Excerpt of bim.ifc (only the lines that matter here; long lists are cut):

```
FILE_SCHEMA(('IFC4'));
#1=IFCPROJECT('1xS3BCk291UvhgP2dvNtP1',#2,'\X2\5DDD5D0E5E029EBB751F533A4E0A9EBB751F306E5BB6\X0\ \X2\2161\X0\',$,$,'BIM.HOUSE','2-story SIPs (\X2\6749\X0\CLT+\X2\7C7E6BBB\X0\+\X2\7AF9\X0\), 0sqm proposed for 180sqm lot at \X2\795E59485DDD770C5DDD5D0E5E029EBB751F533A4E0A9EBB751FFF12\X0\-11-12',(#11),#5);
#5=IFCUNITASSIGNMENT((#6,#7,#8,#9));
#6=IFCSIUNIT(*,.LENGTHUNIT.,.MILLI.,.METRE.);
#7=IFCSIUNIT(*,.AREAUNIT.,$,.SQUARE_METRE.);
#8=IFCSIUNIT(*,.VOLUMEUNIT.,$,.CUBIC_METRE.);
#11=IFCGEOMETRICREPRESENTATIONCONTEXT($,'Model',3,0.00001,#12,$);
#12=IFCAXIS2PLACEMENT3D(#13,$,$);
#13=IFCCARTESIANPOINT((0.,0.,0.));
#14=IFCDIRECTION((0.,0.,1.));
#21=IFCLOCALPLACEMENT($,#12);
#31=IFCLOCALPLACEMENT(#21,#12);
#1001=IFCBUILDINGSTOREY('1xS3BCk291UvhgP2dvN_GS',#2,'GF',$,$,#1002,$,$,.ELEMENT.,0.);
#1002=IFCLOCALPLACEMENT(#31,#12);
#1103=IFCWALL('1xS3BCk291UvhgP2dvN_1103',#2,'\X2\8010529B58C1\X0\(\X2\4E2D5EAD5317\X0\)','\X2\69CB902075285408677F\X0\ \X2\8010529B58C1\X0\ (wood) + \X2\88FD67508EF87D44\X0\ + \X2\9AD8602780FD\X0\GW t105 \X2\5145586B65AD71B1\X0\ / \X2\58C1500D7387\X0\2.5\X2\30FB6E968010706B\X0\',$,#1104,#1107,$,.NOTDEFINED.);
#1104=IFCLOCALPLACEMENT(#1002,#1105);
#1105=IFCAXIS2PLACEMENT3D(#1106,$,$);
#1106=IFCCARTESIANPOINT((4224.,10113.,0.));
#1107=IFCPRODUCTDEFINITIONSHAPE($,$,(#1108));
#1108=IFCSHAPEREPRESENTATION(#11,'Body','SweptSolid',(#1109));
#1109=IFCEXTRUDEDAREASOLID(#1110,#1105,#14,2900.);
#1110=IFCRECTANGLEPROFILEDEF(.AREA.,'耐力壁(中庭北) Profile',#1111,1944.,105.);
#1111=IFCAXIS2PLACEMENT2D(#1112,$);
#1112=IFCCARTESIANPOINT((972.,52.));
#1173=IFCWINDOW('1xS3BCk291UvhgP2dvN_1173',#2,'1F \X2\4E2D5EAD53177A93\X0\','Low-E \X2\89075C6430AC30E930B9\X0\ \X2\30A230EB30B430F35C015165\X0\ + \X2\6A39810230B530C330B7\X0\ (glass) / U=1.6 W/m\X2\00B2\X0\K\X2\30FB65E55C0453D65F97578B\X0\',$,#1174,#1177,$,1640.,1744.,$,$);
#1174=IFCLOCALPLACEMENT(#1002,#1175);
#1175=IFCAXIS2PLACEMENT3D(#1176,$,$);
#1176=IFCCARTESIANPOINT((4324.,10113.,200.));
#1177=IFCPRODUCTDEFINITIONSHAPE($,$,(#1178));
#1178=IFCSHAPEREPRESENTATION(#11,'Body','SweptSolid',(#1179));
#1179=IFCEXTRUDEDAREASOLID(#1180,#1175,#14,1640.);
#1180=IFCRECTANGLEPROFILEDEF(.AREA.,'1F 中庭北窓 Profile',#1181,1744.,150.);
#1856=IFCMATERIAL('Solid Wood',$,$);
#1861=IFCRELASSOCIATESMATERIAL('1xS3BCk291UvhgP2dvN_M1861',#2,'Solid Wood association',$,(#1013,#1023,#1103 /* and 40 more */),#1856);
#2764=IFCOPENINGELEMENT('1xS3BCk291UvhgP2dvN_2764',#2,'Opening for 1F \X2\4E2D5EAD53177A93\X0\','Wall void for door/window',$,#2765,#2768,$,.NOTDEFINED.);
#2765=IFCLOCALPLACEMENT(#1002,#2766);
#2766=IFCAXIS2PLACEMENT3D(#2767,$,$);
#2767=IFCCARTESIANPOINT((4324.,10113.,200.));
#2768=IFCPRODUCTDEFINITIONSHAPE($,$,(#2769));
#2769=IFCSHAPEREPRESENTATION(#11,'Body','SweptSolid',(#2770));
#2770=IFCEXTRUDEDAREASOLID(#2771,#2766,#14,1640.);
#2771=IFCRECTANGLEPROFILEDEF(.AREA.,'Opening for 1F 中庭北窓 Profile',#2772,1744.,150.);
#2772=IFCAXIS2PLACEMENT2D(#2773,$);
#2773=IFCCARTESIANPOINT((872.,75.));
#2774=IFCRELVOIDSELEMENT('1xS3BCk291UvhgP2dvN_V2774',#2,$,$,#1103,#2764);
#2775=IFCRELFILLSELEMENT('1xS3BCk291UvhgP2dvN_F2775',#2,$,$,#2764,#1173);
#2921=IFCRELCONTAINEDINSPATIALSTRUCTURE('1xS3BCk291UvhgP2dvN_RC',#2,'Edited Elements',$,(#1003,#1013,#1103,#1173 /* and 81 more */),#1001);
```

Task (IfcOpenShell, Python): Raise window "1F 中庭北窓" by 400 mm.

```python
import numpy as np
import ifcopenshell
import ifcopenshell.api.geometry
import ifcopenshell.util.placement
import ifcopenshell.util.unit

model = ifcopenshell.open("bim.ifc")
unit_scale = ifcopenshell.util.unit.calculate_unit_scale(model)

window = model.by_guid("1xS3BCk291UvhgP2dvN_1173")
opening = window.FillsVoids[0].RelatingOpeningElement
dz = 0.4 / unit_scale

shift = np.array([0.0, 0.0, dz])
# The window is not placed relative to its opening, so move both.
for product in (opening, window):
    matrix = ifcopenshell.util.placement.get_local_placement(product.ObjectPlacement)
    matrix[:3, 3] += shift
    ifcopenshell.api.geometry.edit_object_placement(model, product=product, matrix=matrix, is_si=False)

print(f"moved by {dz * unit_scale:+.3f} m")

model.write("bim_edited.ifc")
```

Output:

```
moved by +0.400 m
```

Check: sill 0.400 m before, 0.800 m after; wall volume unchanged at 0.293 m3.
